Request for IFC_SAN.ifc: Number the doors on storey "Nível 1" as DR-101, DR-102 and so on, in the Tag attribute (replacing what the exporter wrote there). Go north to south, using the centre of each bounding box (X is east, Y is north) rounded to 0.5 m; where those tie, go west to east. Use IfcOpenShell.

First a look at what the model holds.

```python
import ifcopenshell
import ifcopenshell.util.element
import ifcopenshell.util.placement

model = ifcopenshell.open("IFC_SAN.ifc")
print(model.schema)
storey = next(s for s in model.by_type("IfcBuildingStorey") if s.Name == "Nível 1")
doors = [e for e in ifcopenshell.util.element.get_decomposition(storey) if e.is_a("IfcDoor")]
for e in sorted(doors, key=lambda e: e.id()):
    origin = ifcopenshell.util.placement.get_local_placement(e.ObjectPlacement)[:3, 3]
    print(e.id(), e.Tag, e.Name, origin.round(2) + 0.0, sep=" | ")
```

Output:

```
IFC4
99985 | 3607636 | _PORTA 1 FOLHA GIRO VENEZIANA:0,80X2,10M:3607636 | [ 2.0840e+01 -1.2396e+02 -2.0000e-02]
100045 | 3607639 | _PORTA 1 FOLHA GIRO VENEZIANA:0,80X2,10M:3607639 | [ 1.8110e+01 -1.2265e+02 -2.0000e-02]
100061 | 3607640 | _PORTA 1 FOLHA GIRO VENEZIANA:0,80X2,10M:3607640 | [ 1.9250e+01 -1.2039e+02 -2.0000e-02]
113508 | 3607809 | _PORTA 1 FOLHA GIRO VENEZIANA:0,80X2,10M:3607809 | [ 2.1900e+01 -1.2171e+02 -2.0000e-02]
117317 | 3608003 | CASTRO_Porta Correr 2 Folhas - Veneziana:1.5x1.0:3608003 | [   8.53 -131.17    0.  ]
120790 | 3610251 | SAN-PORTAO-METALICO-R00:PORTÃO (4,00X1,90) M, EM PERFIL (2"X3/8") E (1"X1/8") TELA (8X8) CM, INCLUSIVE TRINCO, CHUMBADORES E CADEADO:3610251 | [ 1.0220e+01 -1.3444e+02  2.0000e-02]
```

```python
import ifcopenshell
import ifcopenshell.geom
import ifcopenshell.util.element
import ifcopenshell.util.shape

model = ifcopenshell.open("IFC_SAN.ifc")
settings = ifcopenshell.geom.settings()
settings.set("use-world-coords", True)


def centre(element):
    shape = ifcopenshell.geom.create_shape(settings, element)
    return ifcopenshell.util.shape.get_bbox_centroid(shape.geometry)


storey = next(s for s in model.by_type("IfcBuildingStorey") if s.Name == "Nível 1")
doors = [e for e in ifcopenshell.util.element.get_decomposition(storey) if e.is_a("IfcDoor")]

# Insertion points can sit at a corner or the storey origin, so sort by the geometry (in metres).
centres = {e: centre(e) for e in doors}
doors.sort(key=lambda e: (-round(centres[e][1] / 0.5), centres[e][0]))

for i, e in enumerate(doors, start=1):
    number = f"DR-1{i:02d}"
    e.Tag = number
    print(e.id(), number)

model.write("IFC_SAN-out.ifc")
```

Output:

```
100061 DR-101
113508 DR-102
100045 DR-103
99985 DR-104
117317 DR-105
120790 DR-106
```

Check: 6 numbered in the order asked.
